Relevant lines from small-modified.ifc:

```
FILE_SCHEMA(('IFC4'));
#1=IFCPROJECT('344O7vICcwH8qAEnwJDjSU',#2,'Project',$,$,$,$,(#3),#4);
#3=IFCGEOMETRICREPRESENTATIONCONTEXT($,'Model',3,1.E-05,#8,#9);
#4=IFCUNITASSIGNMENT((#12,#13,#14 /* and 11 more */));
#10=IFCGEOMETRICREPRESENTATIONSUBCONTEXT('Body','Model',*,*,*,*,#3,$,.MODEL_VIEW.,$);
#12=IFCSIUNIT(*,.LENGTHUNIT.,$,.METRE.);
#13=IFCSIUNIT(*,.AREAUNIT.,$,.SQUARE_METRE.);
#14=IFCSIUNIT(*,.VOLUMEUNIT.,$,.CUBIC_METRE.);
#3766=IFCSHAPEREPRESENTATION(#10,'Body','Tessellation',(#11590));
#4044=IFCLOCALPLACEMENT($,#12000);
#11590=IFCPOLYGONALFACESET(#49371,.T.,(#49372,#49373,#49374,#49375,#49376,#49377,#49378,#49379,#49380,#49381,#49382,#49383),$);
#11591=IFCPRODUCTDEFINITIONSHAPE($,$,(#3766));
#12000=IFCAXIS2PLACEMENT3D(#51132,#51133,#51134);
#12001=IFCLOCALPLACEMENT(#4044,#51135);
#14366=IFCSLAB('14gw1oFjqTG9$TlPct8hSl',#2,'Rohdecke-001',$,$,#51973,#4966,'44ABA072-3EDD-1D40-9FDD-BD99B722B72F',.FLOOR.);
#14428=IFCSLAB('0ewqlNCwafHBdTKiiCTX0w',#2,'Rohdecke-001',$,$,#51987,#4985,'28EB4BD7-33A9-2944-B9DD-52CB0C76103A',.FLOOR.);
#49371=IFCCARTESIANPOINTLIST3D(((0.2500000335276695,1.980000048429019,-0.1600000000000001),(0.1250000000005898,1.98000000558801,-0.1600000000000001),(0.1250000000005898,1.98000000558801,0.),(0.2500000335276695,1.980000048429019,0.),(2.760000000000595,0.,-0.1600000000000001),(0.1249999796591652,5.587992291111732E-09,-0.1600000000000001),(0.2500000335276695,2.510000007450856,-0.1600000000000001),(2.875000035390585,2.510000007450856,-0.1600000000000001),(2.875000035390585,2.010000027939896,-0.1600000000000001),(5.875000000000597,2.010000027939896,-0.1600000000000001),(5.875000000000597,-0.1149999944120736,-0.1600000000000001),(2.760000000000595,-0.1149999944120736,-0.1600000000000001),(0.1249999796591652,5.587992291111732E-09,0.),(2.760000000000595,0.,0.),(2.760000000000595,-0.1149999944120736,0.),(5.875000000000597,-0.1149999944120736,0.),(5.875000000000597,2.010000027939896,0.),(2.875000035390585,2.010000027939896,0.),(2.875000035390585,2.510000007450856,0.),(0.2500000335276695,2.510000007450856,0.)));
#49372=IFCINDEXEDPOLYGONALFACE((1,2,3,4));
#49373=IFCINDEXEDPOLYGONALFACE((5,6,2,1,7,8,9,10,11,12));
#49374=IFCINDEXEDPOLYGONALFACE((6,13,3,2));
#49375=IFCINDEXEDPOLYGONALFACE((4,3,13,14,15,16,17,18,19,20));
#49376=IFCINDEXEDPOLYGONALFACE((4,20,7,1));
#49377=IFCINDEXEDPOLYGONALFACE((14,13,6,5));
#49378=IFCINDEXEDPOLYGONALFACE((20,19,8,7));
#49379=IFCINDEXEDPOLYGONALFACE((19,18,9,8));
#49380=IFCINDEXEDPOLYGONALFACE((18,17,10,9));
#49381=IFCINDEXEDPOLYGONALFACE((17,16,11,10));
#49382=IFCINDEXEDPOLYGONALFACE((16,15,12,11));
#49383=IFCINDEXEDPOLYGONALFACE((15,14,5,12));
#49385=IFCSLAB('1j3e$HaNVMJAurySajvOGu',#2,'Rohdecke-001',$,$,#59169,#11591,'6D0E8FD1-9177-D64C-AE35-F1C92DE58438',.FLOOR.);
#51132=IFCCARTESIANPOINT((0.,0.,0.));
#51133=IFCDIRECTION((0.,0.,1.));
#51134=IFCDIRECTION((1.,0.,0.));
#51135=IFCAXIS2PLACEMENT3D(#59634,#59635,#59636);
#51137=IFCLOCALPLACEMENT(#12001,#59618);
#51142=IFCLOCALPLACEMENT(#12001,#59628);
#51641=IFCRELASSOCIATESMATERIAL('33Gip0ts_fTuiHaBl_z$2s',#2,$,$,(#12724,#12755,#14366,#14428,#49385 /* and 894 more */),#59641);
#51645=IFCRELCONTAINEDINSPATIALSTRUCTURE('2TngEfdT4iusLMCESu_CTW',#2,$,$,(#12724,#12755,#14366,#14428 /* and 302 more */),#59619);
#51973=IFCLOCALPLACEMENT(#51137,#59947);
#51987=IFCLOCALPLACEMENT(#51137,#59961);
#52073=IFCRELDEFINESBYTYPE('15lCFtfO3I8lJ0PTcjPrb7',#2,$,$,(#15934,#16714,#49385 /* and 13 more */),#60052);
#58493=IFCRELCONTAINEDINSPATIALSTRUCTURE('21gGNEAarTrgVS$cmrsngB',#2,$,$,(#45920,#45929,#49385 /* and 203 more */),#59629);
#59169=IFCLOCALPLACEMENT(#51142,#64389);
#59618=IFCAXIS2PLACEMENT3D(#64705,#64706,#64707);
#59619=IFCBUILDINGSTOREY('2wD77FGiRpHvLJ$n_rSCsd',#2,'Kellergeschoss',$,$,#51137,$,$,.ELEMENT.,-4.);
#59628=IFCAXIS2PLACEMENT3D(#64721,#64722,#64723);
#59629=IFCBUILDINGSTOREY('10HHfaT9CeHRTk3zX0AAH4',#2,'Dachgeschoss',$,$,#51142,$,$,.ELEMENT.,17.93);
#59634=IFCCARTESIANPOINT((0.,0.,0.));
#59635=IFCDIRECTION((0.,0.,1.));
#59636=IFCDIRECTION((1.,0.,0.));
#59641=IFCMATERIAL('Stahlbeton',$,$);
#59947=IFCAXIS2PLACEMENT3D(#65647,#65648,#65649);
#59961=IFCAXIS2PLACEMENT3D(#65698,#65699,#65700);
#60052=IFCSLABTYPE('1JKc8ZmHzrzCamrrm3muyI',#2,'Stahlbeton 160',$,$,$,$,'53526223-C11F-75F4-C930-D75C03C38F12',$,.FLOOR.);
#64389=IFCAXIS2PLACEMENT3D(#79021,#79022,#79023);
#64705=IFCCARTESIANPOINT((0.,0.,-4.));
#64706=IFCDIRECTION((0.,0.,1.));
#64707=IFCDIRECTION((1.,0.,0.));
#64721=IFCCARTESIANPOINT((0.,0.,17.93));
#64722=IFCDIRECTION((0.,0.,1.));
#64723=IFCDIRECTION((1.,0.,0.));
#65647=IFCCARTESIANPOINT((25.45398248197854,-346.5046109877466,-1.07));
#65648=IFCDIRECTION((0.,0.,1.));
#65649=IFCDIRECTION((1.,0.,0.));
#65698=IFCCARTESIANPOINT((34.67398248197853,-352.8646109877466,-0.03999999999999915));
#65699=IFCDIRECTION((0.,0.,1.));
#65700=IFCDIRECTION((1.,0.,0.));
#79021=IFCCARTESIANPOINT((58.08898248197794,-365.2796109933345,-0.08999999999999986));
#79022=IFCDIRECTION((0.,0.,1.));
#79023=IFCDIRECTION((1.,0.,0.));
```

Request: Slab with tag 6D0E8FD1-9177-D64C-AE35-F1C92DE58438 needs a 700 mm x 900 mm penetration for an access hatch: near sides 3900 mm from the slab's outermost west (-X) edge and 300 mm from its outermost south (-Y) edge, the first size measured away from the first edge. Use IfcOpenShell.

```python
import numpy as np
import ifcopenshell
import ifcopenshell.api.feature
import ifcopenshell.api.geometry
import ifcopenshell.api.root
import ifcopenshell.geom
import ifcopenshell.util.placement
import ifcopenshell.util.representation
import ifcopenshell.util.shape
import ifcopenshell.util.unit

model = ifcopenshell.open("small-modified.ifc")
unit_scale = ifcopenshell.util.unit.calculate_unit_scale(model)
settings = ifcopenshell.geom.settings()


def volume(element):
    """Net volume in cubic metres, openings subtracted."""
    shape = ifcopenshell.geom.create_shape(settings, element)
    return ifcopenshell.util.shape.get_volume(shape.geometry)


slab = model.by_guid("1j3e$HaNVMJAurySajvOGu")
before = volume(slab)

# Extent in the slab's own axes, in metres. The edges named are its -X and -Y sides.
slab_shape = ifcopenshell.geom.create_shape(settings, slab)
vertices = ifcopenshell.util.shape.get_vertices(slab_shape.geometry)
x_min, y_min, bottom = vertices.min(axis=0)
top = vertices[:, 2].max()

opening = ifcopenshell.api.root.create_entity(model, ifc_class="IfcOpeningElement", name="Access hatch opening", predefined_type="OPENING")
context = ifcopenshell.util.representation.get_context(model, "Model", "Body", "MODEL_VIEW")
width, depth = 0.7, 0.9
outline = [(0.0, 0.0), (width, 0.0), (width, depth), (0.0, depth), (0.0, 0.0)]
# Overshoot both faces by 50 mm so the cut is clean.
shape = ifcopenshell.api.geometry.add_slab_representation(
    model, context=context, depth=top - bottom + 0.1, polyline=outline
)
ifcopenshell.api.geometry.assign_representation(model, product=opening, representation=shape)

matrix = ifcopenshell.util.placement.get_local_placement(slab.ObjectPlacement)
matrix[:, 3] = matrix @ np.append(np.array([x_min + 3.9, y_min + 0.3, bottom - 0.05]) / unit_scale, 1.0)
ifcopenshell.api.geometry.edit_object_placement(model, product=opening, matrix=matrix, is_si=False)
ifcopenshell.api.feature.add_feature(model, feature=opening, element=slab)

after = volume(slab)

print(f"slab volume {before:.3f} -> {after:.3f} m3")

model.write("small-modified_updated.ifc")
```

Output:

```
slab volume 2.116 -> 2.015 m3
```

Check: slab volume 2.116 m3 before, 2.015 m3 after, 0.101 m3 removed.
